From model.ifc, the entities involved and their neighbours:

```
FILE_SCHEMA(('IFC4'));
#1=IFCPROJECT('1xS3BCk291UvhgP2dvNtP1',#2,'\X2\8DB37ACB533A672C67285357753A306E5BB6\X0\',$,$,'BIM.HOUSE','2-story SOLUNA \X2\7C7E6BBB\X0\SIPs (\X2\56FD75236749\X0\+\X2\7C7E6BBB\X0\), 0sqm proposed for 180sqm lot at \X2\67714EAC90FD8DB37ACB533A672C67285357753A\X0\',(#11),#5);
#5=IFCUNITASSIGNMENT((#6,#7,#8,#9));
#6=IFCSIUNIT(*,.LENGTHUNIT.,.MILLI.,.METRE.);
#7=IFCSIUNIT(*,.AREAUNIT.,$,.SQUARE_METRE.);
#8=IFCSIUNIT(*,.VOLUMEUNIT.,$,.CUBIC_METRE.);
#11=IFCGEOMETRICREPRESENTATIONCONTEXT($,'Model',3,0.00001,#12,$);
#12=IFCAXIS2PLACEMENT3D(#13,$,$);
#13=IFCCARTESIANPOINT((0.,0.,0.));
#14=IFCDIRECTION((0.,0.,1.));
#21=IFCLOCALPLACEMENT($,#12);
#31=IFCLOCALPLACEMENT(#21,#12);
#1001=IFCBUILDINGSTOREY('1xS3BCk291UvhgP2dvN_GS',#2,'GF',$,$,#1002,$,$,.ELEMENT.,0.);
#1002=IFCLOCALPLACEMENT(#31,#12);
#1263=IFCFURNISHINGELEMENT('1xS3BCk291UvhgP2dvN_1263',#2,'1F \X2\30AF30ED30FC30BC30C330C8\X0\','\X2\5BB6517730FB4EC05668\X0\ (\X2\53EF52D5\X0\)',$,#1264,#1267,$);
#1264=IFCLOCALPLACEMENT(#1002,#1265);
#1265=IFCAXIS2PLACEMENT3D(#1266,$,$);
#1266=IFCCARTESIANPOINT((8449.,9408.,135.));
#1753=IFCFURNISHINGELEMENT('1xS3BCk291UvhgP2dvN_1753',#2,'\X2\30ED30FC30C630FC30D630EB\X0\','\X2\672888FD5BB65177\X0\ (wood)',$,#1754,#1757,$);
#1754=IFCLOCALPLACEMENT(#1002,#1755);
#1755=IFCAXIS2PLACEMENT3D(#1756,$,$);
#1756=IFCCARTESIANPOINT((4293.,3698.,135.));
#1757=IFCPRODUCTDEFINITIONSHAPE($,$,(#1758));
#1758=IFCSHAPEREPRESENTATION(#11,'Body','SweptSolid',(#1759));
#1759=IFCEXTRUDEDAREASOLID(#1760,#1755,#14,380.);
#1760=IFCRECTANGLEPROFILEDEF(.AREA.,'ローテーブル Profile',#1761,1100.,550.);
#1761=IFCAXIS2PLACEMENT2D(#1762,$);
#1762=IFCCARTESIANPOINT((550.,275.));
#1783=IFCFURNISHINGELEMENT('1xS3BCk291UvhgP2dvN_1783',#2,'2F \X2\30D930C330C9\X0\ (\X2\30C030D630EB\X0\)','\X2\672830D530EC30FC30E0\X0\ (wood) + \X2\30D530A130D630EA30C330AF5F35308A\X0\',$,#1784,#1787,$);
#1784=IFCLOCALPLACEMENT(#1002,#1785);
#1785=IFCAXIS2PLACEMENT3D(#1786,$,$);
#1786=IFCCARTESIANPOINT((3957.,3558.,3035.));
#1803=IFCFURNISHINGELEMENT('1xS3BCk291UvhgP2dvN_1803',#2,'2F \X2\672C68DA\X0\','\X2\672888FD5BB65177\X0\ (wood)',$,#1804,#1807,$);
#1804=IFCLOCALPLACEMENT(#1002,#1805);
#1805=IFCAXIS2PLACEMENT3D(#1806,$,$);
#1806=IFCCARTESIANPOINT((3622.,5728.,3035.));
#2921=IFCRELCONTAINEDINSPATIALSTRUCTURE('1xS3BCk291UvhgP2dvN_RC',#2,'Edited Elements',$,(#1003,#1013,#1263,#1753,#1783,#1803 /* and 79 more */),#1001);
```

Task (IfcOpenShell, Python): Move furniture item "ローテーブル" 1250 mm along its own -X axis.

```python
import ifcopenshell
import ifcopenshell.api.geometry
import ifcopenshell.util.placement
import ifcopenshell.util.unit

model = ifcopenshell.open("model.ifc")
unit_scale = ifcopenshell.util.unit.calculate_unit_scale(model)

item = model.by_guid("1xS3BCk291UvhgP2dvN_1753")
matrix = ifcopenshell.util.placement.get_local_placement(item.ObjectPlacement)
matrix[:3, 3] -= matrix[:3, 0] * 1.25 / unit_scale
ifcopenshell.api.geometry.edit_object_placement(model, product=item, matrix=matrix, is_si=False)

print(ifcopenshell.util.placement.get_local_placement(item.ObjectPlacement).round(3) + 0.0)

model.write("model_v2.ifc")
```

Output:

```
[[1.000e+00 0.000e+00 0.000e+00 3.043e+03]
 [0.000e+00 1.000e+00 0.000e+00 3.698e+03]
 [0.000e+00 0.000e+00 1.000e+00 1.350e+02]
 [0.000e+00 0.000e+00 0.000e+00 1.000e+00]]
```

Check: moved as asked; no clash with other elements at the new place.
